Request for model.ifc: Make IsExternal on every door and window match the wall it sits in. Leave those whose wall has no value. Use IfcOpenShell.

First a look at what the model holds.

```python
import ifcopenshell
import ifcopenshell.util.element

model = ifcopenshell.open("model.ifc")
print(model.schema)
seen = {}
for e in model.by_type("IfcDoor") + model.by_type("IfcWindow"):
    if not e.FillsVoids:
        continue
    host = e.FillsVoids[0].RelatingOpeningElement.VoidsElements[0].RelatingBuildingElement
    own = ifcopenshell.util.element.get_pset(e, f"Pset_{e.is_a()[3:].removesuffix('StandardCase')}Common", "IsExternal")
    wall = ifcopenshell.util.element.get_pset(host, "Pset_WallCommon", "IsExternal")
    seen[e.is_a(), own, wall] = seen.get((e.is_a(), own, wall), 0) + 1
for (cls, own, wall), count in sorted(seen.items(), key=str):
    print(count, cls, "IsExternal:", own, "| host wall:", wall)
```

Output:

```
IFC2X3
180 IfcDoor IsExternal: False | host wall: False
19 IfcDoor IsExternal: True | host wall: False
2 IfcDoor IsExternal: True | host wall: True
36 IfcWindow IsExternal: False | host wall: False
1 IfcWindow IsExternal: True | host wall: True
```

```python
import ifcopenshell
import ifcopenshell.api.pset
import ifcopenshell.util.element

model = ifcopenshell.open("model.ifc")

count = 0
for ifc_class, pset_name in (("IfcDoor", "Pset_DoorCommon"), ("IfcWindow", "Pset_WindowCommon")):
    for e in model.by_type(ifc_class):
        if not e.FillsVoids:
            continue
        host = e.FillsVoids[0].RelatingOpeningElement.VoidsElements[0].RelatingBuildingElement
        external = ifcopenshell.util.element.get_pset(host, "Pset_WallCommon", "IsExternal")
        if external is None or ifcopenshell.util.element.get_pset(e, pset_name, "IsExternal") == external:
            continue
        pset = ifcopenshell.api.pset.add_pset(model, product=e, name=pset_name)
        ifcopenshell.api.pset.edit_pset(model, pset=pset, properties={"IsExternal": external})
        count += 1

print(count, "updated")

model.write("model_updated.ifc")
```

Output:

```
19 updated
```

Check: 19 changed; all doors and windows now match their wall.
